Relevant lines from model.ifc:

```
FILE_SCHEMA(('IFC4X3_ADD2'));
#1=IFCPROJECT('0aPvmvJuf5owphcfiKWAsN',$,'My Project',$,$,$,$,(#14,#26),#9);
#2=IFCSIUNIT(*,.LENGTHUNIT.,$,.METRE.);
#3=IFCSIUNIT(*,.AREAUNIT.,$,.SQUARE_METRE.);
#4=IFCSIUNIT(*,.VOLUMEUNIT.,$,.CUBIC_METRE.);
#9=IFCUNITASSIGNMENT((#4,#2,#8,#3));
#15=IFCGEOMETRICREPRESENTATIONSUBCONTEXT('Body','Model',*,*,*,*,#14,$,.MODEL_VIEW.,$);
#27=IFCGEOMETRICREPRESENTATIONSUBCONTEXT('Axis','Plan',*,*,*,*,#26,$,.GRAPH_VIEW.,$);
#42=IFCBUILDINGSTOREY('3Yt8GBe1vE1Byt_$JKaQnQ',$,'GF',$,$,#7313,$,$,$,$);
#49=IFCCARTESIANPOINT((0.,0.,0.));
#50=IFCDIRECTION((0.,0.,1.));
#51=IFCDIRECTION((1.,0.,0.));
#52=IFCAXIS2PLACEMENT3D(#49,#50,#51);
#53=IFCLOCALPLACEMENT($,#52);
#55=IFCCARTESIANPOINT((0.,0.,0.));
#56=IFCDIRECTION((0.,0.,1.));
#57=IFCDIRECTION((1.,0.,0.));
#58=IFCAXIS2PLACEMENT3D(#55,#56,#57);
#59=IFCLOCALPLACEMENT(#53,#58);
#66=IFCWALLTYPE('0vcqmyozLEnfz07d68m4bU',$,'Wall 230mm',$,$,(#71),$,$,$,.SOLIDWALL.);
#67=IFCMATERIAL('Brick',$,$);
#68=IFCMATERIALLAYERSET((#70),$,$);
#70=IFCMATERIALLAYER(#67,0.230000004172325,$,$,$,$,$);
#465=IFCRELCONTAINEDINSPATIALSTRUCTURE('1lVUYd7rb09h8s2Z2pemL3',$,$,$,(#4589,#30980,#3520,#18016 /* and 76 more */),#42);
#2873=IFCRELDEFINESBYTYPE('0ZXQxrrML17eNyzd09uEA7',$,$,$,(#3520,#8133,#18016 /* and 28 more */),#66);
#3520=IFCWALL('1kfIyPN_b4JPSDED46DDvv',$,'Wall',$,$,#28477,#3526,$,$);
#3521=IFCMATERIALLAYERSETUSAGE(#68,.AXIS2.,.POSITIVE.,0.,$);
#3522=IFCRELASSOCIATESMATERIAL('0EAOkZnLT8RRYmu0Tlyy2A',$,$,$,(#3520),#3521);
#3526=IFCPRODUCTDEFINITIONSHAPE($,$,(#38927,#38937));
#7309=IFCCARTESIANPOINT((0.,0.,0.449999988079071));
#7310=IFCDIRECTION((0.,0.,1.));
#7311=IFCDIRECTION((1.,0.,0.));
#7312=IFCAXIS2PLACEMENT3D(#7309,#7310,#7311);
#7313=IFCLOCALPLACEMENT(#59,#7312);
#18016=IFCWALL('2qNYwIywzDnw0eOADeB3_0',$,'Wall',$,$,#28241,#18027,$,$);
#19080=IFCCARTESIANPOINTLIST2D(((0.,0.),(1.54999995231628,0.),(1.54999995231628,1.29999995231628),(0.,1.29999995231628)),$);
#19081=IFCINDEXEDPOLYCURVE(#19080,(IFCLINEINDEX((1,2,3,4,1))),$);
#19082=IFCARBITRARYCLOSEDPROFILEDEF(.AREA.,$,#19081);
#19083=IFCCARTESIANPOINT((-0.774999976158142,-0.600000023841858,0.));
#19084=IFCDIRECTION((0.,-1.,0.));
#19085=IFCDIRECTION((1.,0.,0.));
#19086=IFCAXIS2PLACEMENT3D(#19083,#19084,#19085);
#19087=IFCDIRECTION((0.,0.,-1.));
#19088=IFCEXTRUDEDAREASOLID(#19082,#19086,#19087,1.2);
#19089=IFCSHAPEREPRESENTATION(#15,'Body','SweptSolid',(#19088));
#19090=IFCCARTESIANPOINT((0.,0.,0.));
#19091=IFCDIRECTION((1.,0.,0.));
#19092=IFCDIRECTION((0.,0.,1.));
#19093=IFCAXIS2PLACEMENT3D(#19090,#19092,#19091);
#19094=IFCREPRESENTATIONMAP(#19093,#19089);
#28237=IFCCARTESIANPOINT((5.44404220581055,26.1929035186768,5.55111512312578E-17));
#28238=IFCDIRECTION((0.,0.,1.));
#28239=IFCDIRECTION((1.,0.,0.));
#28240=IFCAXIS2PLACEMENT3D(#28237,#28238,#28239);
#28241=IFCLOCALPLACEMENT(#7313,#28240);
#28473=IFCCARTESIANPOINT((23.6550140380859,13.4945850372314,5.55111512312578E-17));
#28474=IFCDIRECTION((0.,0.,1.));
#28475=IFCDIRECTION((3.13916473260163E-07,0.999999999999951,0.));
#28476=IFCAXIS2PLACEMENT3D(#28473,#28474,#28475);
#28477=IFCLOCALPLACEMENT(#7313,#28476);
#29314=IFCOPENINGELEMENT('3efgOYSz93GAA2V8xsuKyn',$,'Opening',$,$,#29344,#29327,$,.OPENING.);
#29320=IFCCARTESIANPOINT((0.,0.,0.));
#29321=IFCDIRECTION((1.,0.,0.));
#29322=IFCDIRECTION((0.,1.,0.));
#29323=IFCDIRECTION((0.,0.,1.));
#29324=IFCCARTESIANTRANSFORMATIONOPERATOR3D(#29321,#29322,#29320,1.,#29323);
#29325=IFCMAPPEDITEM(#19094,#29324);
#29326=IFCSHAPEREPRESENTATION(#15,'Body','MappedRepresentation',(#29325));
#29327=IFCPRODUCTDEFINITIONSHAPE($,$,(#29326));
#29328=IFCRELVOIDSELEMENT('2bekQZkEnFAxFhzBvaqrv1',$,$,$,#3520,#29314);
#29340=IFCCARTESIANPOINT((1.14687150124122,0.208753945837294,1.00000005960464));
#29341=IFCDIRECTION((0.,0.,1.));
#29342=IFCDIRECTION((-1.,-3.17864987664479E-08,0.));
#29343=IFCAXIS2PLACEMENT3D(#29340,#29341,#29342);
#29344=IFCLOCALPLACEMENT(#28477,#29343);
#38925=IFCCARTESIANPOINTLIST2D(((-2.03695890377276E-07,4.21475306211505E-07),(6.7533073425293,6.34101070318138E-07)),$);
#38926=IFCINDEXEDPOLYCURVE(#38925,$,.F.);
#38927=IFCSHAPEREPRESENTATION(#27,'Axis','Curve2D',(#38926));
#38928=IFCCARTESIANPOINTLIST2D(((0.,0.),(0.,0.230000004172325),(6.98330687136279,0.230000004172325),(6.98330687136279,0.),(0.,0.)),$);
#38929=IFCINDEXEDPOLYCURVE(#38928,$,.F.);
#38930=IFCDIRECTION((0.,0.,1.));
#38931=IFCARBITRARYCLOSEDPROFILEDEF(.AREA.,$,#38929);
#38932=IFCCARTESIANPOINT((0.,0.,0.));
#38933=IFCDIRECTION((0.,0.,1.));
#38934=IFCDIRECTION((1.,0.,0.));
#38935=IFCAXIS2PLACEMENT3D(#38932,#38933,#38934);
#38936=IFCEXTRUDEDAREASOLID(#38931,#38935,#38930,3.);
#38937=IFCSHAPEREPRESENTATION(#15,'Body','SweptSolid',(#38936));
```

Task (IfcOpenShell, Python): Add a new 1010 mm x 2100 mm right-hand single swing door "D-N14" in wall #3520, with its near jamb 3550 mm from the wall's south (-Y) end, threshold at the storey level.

```python
import numpy as np
import ifcopenshell
import ifcopenshell.api.feature
import ifcopenshell.api.geometry
import ifcopenshell.api.root
import ifcopenshell.api.spatial
import ifcopenshell.geom
import ifcopenshell.util.element
import ifcopenshell.util.placement
import ifcopenshell.util.representation
import ifcopenshell.util.shape
import ifcopenshell.util.unit

model = ifcopenshell.open("model.ifc")
unit_scale = ifcopenshell.util.unit.calculate_unit_scale(model)
settings = ifcopenshell.geom.settings()


def volume(element):
    """Net volume in cubic metres, openings subtracted."""
    shape = ifcopenshell.geom.create_shape(settings, element)
    return ifcopenshell.util.shape.get_volume(shape.geometry)


wall = model.by_guid("1kfIyPN_b4JPSDED46DDvv")
storey = ifcopenshell.util.element.get_container(wall, ifc_class="IfcBuildingStorey")
context = ifcopenshell.util.representation.get_context(model, "Model", "Body", "MODEL_VIEW")
before = volume(wall)

width, height, from_end, sill = 1.01, 2.1, 3.55, 0.0  # metres

# The wall runs along its own X axis, and the end named is its -X end.
wall_shape = ifcopenshell.geom.create_shape(settings, wall)
x, y, z = ifcopenshell.util.shape.get_vertices(wall_shape.geometry).T
start = x.min() + from_end
face, thickness = float(y.min()), float(y.max() - y.min())
wall_matrix = ifcopenshell.util.placement.get_local_placement(wall.ObjectPlacement)
level = ifcopenshell.util.placement.get_local_placement(storey.ObjectPlacement)[2, 3]


def in_wall(x, y):
    """Placement at x, y metres in the wall's axes, at sill height."""
    matrix = wall_matrix.copy()
    matrix[:, 3] = wall_matrix @ np.array([x / unit_scale, y / unit_scale, 0.0, 1.0])
    matrix[2, 3] = level + sill / unit_scale
    return matrix


# Opening: a box that overshoots both wall faces by 50 mm.
opening = ifcopenshell.api.root.create_entity(model, ifc_class="IfcOpeningElement", predefined_type="OPENING")
box = ifcopenshell.api.geometry.add_wall_representation(
    model, context=context, length=width, height=height, thickness=thickness + 0.1
)
ifcopenshell.api.geometry.assign_representation(model, product=opening, representation=box)
ifcopenshell.api.geometry.edit_object_placement(model, product=opening, matrix=in_wall(start, face - 0.05), is_si=False)
ifcopenshell.api.feature.add_feature(model, feature=opening, element=wall)

door = ifcopenshell.api.root.create_entity(model, ifc_class="IfcDoor", name="D-N14", predefined_type="DOOR")
door.OverallWidth, door.OverallHeight = width / unit_scale, height / unit_scale
door.OperationType = "SINGLE_SWING_RIGHT"
body = ifcopenshell.api.geometry.add_door_representation(
    model,
    context=context,
    overall_width=door.OverallWidth,
    overall_height=door.OverallHeight,
    operation_type="SINGLE_SWING_RIGHT",
    lining_properties={"LiningDepth": thickness / unit_scale, "ThresholdDepth": thickness / unit_scale},
)
ifcopenshell.api.geometry.assign_representation(model, product=door, representation=body)
ifcopenshell.api.spatial.assign_container(model, products=[door], relating_structure=storey)
ifcopenshell.api.feature.add_filling(model, opening=opening, element=door)

# The lining spans the wall, so the door starts at the wall face.
ifcopenshell.api.geometry.edit_object_placement(model, product=door, matrix=in_wall(start, face), is_si=False)

after = volume(wall)

print(f"wall volume {before:.3f} -> {after:.3f} m3")

model.write("model_edited.ifc")
```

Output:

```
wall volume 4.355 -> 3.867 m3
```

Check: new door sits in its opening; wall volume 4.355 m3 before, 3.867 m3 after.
